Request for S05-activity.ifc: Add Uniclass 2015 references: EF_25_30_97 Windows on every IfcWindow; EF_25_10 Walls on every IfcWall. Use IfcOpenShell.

First a look at what the model holds.

```python
import ifcopenshell

model = ifcopenshell.open("S05-activity.ifc")
print(model.schema)
print("classifications:", [c.Name for c in model.by_type("IfcClassification")])
for ifc_class in ("IfcDoor", "IfcRoof", "IfcStair", "IfcWall", "IfcWindow"):
    print(ifc_class, len(model.by_type(ifc_class)))
```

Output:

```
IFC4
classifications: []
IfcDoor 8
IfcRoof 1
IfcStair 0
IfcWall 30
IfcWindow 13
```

```python
import ifcopenshell
import ifcopenshell.api.classification

model = ifcopenshell.open("S05-activity.ifc")

system = ifcopenshell.api.classification.add_classification(model, classification="Uniclass 2015")

codes = {
    "IfcWindow": ("EF_25_30_97", "Windows"),
    "IfcWall": ("EF_25_10", "Walls"),
}
for ifc_class, (code, name) in codes.items():
    products = model.by_type(ifc_class)
    ifcopenshell.api.classification.add_reference(
        model, products=products, classification=system, identification=code, name=name
    )
    print(code, len(products))

model.write("S05-activity_v2.ifc")
```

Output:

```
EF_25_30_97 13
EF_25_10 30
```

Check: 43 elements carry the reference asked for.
